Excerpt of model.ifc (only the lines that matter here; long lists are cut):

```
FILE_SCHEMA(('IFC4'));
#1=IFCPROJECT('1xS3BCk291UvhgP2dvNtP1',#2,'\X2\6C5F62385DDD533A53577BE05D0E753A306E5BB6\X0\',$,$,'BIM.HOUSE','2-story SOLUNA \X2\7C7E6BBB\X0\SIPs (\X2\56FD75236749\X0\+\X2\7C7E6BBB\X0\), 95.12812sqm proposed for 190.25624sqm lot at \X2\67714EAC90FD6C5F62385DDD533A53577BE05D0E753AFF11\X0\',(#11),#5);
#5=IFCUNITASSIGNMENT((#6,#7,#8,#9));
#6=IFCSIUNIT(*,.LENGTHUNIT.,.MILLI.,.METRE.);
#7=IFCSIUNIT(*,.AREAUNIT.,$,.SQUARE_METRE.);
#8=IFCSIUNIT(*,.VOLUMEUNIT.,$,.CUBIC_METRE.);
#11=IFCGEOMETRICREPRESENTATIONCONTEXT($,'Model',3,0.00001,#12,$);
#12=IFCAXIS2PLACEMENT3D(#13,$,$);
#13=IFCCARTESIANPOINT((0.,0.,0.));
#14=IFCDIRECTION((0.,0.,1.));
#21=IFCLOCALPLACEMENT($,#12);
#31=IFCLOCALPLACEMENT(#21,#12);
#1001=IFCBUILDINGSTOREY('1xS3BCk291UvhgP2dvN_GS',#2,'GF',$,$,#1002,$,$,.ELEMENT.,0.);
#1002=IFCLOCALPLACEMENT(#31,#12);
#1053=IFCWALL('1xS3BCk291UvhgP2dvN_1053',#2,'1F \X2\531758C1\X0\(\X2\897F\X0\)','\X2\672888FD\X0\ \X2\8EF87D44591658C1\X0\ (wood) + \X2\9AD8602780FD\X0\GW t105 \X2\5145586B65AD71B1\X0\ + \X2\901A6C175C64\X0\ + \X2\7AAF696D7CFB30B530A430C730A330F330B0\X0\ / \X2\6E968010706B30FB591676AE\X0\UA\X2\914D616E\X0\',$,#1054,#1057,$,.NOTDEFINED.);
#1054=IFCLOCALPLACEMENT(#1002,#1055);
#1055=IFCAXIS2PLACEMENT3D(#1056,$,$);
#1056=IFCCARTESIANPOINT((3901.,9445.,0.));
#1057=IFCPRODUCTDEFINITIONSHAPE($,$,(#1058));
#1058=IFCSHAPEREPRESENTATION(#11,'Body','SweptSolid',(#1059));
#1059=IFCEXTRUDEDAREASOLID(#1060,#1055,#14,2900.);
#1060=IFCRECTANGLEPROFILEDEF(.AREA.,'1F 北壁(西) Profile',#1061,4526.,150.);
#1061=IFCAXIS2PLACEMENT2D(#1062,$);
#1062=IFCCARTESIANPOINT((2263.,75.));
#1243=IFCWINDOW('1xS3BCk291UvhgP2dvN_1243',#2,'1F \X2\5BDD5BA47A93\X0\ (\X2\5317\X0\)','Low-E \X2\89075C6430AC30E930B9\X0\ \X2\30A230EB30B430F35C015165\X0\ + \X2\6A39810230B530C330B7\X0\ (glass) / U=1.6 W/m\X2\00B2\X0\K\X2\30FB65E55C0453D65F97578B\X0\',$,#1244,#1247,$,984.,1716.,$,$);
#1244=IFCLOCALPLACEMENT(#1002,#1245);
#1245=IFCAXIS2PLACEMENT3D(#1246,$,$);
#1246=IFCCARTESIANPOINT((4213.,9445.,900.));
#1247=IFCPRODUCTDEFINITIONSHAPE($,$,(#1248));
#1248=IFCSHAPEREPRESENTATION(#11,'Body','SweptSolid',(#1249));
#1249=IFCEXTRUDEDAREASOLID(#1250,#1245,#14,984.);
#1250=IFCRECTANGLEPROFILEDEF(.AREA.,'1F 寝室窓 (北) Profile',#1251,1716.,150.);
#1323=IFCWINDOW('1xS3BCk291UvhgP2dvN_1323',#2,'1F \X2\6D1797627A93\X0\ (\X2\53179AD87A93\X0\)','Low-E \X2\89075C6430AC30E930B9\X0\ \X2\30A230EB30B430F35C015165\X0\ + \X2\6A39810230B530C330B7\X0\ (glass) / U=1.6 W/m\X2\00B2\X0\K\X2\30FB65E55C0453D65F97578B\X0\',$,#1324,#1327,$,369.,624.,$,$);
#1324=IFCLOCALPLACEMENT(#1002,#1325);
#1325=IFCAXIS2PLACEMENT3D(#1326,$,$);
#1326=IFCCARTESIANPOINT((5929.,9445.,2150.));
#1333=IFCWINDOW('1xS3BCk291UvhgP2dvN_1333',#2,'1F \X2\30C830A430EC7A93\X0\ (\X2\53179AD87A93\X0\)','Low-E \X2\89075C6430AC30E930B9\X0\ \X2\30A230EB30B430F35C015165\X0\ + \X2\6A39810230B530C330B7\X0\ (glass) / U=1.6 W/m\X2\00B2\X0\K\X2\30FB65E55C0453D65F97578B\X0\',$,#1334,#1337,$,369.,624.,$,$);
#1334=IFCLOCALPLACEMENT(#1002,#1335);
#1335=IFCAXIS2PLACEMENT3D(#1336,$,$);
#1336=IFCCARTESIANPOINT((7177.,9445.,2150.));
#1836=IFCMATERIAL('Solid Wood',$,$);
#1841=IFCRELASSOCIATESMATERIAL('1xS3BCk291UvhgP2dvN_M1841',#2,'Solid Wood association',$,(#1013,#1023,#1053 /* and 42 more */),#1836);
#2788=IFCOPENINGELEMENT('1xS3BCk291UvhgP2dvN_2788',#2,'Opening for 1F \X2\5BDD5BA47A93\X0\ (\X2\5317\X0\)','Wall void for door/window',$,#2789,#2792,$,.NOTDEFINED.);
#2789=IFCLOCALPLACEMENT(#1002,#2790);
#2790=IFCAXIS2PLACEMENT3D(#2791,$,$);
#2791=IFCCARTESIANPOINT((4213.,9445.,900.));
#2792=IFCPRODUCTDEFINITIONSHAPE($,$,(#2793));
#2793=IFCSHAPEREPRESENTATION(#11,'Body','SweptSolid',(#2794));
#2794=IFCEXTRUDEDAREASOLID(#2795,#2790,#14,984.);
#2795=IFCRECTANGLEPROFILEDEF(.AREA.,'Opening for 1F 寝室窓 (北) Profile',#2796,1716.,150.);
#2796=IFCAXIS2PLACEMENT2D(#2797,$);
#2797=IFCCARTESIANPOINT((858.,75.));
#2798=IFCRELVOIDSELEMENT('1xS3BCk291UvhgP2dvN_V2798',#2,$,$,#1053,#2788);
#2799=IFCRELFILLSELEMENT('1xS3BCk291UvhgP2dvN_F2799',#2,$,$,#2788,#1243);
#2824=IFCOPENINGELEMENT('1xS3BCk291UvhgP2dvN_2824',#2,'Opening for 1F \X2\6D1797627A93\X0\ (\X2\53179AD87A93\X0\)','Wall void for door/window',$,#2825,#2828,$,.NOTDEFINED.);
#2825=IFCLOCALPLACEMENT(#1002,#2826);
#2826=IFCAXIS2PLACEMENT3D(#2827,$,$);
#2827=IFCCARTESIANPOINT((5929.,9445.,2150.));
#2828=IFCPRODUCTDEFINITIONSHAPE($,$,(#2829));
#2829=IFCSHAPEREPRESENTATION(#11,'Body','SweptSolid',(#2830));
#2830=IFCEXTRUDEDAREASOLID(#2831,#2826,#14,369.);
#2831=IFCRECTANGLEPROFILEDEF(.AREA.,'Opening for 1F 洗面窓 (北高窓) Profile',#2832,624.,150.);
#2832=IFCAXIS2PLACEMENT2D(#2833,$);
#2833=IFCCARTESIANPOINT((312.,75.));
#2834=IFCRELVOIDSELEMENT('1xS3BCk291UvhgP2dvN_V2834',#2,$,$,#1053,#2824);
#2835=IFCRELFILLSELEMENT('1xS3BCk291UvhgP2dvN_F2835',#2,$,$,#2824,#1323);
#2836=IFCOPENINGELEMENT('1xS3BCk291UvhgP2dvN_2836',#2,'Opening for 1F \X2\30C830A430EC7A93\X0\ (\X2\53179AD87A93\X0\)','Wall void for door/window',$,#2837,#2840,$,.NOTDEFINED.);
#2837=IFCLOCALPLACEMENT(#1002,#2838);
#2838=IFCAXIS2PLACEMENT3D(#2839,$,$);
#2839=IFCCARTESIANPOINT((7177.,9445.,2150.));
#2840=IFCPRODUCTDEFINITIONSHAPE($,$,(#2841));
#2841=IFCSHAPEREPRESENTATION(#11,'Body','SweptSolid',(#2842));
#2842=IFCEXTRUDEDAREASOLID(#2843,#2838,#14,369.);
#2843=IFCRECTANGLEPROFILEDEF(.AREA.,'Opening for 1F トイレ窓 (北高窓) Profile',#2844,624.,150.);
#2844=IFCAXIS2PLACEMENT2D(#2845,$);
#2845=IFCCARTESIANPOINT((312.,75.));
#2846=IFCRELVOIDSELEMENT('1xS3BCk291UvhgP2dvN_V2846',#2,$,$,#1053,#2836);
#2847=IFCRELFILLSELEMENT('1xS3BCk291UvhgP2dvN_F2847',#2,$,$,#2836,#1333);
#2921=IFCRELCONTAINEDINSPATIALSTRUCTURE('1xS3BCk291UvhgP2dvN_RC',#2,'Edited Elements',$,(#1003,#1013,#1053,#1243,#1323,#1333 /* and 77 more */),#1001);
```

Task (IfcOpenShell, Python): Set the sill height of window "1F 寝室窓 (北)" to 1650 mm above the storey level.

```python
import numpy as np
import ifcopenshell
import ifcopenshell.api.geometry
import ifcopenshell.geom
import ifcopenshell.util.element
import ifcopenshell.util.placement
import ifcopenshell.util.shape
import ifcopenshell.util.unit

model = ifcopenshell.open("model.ifc")
unit_scale = ifcopenshell.util.unit.calculate_unit_scale(model)

window = model.by_id(1243)
opening = window.FillsVoids[0].RelatingOpeningElement
storey = ifcopenshell.util.element.get_container(window, ifc_class="IfcBuildingStorey")
level = ifcopenshell.util.placement.get_local_placement(storey.ObjectPlacement)[2, 3]

# The opening's origin need not be at the sill, so measure its lowest point.
shape = ifcopenshell.geom.create_shape(ifcopenshell.geom.settings(), opening)
bottom = ifcopenshell.util.shape.get_shape_bottom_elevation(shape, shape.geometry) / unit_scale
dz = level + 1650.0 - bottom

shift = np.array([0.0, 0.0, dz])
# The window is not placed relative to its opening, so move both.
for product in (opening, window):
    matrix = ifcopenshell.util.placement.get_local_placement(product.ObjectPlacement)
    matrix[:3, 3] += shift
    ifcopenshell.api.geometry.edit_object_placement(model, product=product, matrix=matrix, is_si=False)

print(f"moved by {dz * unit_scale:+.3f} m")

model.write("model_edited.ifc")
```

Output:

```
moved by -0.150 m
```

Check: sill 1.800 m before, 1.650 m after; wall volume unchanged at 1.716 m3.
